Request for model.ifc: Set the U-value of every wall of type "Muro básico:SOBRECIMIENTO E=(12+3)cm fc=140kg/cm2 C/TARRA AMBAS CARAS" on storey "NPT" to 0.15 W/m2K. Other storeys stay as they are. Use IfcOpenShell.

First a look at what the model holds.

```python
import ifcopenshell
import ifcopenshell.util.element

model = ifcopenshell.open("model.ifc")
print(model.schema)
storey = next(s for s in model.by_type("IfcBuildingStorey") if s.Name == "NPT")
walls = [e for e in ifcopenshell.util.element.get_decomposition(storey) if e.is_a("IfcWall")]
seen = {}
for e in walls:
    element_type = ifcopenshell.util.element.get_type(e)
    key = (element_type.Name if element_type != e and element_type else None, ifcopenshell.util.element.get_pset(e, "Pset_WallCommon", "ThermalTransmittance"))
    seen[key] = seen.get(key, 0) + 1
for (name, value), count in sorted(seen.items(), key=str):
    print(count, "x", name, "|", value)
```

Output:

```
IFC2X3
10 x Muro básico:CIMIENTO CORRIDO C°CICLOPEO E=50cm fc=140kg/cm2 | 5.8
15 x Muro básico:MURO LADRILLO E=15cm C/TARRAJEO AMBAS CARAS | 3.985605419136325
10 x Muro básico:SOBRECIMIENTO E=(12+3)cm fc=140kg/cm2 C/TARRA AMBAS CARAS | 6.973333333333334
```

```python
import ifcopenshell
import ifcopenshell.api.pset
import ifcopenshell.util.element

model = ifcopenshell.open("model.ifc")

storey = next(s for s in model.by_type("IfcBuildingStorey") if s.Name == "NPT")
walls = [e for e in ifcopenshell.util.element.get_decomposition(storey) if e.is_a("IfcWall")]

count = 0
for e in walls:
    element_type = ifcopenshell.util.element.get_type(e)
    if element_type in (None, e) or element_type.Name != "Muro básico:SOBRECIMIENTO E=(12+3)cm fc=140kg/cm2 C/TARRA AMBAS CARAS":
        continue
    # add_pset returns the element's existing set when there is one.
    pset = ifcopenshell.api.pset.add_pset(model, product=e, name="Pset_WallCommon")
    ifcopenshell.api.pset.edit_pset(model, pset=pset, properties={"ThermalTransmittance": 0.15})
    count += 1

print(count, "walls updated")

model.write("model_edited.ifc")
```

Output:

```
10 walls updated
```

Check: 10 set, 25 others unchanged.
